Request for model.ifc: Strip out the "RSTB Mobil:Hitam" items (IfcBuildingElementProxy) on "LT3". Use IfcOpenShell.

First a look at what the model holds.

```python
import ifcopenshell
import ifcopenshell.util.element

model = ifcopenshell.open("model.ifc")
print(model.schema)
storey = next(s for s in model.by_type("IfcBuildingStorey") if s.Name == "LT3")
proxies = [e for e in ifcopenshell.util.element.get_decomposition(storey) if e.is_a("IfcBuildingElementProxy")]
seen = {}
for e in proxies:
    element_type = ifcopenshell.util.element.get_type(e)
    name = element_type.Name if element_type not in (None, e) else None
    seen[name] = seen.get(name, 0) + 1
for name, count in sorted(seen.items(), key=str):
    print(count, "x", name)
```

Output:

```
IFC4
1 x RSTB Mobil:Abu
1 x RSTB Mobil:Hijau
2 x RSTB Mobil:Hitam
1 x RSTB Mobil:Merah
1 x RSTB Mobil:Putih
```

```python
import ifcopenshell
import ifcopenshell.api.root
import ifcopenshell.util.element

model = ifcopenshell.open("model.ifc")

storey = next(s for s in model.by_type("IfcBuildingStorey") if s.Name == "LT3")
proxies = [e for e in ifcopenshell.util.element.get_decomposition(storey) if e.is_a("IfcBuildingElementProxy")]
targets = [e for e in proxies if (t := ifcopenshell.util.element.get_type(e)) not in (None, e) and t.Name == "RSTB Mobil:Hitam"]

for e in targets:
    ifcopenshell.api.root.remove_product(model, product=e)
print(len(targets), "removed")

model.write("model_edited.ifc")
```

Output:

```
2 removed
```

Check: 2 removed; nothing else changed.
